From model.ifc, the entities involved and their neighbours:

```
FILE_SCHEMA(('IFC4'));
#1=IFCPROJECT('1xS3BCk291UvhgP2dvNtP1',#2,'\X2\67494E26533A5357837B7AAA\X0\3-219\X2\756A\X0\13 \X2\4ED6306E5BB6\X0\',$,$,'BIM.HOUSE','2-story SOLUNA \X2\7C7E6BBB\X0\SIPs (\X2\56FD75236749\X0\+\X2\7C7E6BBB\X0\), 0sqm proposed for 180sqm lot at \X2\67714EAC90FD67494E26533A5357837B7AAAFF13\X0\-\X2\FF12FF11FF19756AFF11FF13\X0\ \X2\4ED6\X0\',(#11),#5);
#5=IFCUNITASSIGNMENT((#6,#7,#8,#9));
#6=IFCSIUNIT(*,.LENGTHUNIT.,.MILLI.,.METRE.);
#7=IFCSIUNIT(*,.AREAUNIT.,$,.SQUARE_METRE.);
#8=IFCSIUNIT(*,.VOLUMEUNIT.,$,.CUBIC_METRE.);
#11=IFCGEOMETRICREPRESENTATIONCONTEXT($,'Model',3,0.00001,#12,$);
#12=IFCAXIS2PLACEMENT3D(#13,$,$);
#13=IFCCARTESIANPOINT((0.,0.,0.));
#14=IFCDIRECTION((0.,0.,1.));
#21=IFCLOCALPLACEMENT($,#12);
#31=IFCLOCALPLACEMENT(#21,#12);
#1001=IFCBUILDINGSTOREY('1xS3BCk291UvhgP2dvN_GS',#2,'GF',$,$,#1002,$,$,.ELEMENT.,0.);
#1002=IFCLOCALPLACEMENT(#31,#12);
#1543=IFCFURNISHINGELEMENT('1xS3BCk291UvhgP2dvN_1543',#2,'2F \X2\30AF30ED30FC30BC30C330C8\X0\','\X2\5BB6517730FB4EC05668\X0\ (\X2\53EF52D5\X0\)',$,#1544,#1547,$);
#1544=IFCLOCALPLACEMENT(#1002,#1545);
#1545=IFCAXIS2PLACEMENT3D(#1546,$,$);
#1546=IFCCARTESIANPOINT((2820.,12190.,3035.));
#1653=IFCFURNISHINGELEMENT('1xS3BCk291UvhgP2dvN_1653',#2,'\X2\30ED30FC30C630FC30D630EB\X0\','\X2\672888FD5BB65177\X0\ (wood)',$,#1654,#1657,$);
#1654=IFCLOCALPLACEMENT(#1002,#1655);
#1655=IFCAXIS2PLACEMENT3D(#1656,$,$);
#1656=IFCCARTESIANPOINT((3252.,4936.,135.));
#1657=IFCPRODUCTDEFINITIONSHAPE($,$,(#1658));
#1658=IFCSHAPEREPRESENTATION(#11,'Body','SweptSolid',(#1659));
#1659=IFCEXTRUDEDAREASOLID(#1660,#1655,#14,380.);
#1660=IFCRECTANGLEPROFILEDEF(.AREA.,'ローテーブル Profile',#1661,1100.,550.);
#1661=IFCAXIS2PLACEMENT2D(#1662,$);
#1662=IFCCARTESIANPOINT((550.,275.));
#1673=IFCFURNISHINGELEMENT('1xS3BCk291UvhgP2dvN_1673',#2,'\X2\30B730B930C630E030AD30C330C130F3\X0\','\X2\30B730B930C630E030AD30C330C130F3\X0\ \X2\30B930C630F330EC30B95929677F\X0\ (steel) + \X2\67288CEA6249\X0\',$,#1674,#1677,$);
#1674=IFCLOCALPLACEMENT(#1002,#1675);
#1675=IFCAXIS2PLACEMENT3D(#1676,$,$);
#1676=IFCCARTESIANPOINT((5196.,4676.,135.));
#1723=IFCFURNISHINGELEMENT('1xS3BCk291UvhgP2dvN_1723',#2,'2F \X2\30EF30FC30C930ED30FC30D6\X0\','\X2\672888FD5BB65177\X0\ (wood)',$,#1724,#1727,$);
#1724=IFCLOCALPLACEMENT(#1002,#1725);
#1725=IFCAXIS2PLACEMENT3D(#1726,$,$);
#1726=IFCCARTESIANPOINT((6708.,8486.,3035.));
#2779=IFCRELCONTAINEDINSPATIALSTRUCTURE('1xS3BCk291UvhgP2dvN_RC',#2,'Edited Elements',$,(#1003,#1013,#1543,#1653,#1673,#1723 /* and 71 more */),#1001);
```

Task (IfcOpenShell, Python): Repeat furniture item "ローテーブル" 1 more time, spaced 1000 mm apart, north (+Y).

```python
import numpy as np
import ifcopenshell
import ifcopenshell.api.geometry
import ifcopenshell.api.root
import ifcopenshell.util.element
import ifcopenshell.util.placement
import ifcopenshell.util.unit

model = ifcopenshell.open("model.ifc")
unit_scale = ifcopenshell.util.unit.calculate_unit_scale(model)


def reuse_history(source, copy):
    """copy_class also copies each property set's owner history, people and application; keep the originals."""
    for rel in copy.IsDefinedBy:
        if rel.is_a("IfcRelDefinesByProperties") and (history := rel.RelatingPropertyDefinition.OwnerHistory):
            rel.RelatingPropertyDefinition.OwnerHistory = source.OwnerHistory
            ifcopenshell.util.element.remove_deep2(model, history)


source = model.by_guid("1xS3BCk291UvhgP2dvN_1653")
base = ifcopenshell.util.placement.get_local_placement(source.ObjectPlacement)
step = np.array([0.0, 1.0, 0.0]) * 1 / unit_scale

for i in range(1, 2):
    copy = ifcopenshell.api.root.copy_class(model, product=source)
    copy.Representation = ifcopenshell.util.element.copy_deep(
        model, source.Representation, exclude=["IfcGeometricRepresentationContext", "IfcRepresentationMap"]
    )
    reuse_history(source, copy)
    matrix = base.copy()
    matrix[:3, 3] += i * step
    print("added at", matrix[:3, 3].round(3) + 0.0)
    ifcopenshell.api.geometry.edit_object_placement(model, product=copy, matrix=matrix, is_si=False)

model.write("model_edited.ifc")
```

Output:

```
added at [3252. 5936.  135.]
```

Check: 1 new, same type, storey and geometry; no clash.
